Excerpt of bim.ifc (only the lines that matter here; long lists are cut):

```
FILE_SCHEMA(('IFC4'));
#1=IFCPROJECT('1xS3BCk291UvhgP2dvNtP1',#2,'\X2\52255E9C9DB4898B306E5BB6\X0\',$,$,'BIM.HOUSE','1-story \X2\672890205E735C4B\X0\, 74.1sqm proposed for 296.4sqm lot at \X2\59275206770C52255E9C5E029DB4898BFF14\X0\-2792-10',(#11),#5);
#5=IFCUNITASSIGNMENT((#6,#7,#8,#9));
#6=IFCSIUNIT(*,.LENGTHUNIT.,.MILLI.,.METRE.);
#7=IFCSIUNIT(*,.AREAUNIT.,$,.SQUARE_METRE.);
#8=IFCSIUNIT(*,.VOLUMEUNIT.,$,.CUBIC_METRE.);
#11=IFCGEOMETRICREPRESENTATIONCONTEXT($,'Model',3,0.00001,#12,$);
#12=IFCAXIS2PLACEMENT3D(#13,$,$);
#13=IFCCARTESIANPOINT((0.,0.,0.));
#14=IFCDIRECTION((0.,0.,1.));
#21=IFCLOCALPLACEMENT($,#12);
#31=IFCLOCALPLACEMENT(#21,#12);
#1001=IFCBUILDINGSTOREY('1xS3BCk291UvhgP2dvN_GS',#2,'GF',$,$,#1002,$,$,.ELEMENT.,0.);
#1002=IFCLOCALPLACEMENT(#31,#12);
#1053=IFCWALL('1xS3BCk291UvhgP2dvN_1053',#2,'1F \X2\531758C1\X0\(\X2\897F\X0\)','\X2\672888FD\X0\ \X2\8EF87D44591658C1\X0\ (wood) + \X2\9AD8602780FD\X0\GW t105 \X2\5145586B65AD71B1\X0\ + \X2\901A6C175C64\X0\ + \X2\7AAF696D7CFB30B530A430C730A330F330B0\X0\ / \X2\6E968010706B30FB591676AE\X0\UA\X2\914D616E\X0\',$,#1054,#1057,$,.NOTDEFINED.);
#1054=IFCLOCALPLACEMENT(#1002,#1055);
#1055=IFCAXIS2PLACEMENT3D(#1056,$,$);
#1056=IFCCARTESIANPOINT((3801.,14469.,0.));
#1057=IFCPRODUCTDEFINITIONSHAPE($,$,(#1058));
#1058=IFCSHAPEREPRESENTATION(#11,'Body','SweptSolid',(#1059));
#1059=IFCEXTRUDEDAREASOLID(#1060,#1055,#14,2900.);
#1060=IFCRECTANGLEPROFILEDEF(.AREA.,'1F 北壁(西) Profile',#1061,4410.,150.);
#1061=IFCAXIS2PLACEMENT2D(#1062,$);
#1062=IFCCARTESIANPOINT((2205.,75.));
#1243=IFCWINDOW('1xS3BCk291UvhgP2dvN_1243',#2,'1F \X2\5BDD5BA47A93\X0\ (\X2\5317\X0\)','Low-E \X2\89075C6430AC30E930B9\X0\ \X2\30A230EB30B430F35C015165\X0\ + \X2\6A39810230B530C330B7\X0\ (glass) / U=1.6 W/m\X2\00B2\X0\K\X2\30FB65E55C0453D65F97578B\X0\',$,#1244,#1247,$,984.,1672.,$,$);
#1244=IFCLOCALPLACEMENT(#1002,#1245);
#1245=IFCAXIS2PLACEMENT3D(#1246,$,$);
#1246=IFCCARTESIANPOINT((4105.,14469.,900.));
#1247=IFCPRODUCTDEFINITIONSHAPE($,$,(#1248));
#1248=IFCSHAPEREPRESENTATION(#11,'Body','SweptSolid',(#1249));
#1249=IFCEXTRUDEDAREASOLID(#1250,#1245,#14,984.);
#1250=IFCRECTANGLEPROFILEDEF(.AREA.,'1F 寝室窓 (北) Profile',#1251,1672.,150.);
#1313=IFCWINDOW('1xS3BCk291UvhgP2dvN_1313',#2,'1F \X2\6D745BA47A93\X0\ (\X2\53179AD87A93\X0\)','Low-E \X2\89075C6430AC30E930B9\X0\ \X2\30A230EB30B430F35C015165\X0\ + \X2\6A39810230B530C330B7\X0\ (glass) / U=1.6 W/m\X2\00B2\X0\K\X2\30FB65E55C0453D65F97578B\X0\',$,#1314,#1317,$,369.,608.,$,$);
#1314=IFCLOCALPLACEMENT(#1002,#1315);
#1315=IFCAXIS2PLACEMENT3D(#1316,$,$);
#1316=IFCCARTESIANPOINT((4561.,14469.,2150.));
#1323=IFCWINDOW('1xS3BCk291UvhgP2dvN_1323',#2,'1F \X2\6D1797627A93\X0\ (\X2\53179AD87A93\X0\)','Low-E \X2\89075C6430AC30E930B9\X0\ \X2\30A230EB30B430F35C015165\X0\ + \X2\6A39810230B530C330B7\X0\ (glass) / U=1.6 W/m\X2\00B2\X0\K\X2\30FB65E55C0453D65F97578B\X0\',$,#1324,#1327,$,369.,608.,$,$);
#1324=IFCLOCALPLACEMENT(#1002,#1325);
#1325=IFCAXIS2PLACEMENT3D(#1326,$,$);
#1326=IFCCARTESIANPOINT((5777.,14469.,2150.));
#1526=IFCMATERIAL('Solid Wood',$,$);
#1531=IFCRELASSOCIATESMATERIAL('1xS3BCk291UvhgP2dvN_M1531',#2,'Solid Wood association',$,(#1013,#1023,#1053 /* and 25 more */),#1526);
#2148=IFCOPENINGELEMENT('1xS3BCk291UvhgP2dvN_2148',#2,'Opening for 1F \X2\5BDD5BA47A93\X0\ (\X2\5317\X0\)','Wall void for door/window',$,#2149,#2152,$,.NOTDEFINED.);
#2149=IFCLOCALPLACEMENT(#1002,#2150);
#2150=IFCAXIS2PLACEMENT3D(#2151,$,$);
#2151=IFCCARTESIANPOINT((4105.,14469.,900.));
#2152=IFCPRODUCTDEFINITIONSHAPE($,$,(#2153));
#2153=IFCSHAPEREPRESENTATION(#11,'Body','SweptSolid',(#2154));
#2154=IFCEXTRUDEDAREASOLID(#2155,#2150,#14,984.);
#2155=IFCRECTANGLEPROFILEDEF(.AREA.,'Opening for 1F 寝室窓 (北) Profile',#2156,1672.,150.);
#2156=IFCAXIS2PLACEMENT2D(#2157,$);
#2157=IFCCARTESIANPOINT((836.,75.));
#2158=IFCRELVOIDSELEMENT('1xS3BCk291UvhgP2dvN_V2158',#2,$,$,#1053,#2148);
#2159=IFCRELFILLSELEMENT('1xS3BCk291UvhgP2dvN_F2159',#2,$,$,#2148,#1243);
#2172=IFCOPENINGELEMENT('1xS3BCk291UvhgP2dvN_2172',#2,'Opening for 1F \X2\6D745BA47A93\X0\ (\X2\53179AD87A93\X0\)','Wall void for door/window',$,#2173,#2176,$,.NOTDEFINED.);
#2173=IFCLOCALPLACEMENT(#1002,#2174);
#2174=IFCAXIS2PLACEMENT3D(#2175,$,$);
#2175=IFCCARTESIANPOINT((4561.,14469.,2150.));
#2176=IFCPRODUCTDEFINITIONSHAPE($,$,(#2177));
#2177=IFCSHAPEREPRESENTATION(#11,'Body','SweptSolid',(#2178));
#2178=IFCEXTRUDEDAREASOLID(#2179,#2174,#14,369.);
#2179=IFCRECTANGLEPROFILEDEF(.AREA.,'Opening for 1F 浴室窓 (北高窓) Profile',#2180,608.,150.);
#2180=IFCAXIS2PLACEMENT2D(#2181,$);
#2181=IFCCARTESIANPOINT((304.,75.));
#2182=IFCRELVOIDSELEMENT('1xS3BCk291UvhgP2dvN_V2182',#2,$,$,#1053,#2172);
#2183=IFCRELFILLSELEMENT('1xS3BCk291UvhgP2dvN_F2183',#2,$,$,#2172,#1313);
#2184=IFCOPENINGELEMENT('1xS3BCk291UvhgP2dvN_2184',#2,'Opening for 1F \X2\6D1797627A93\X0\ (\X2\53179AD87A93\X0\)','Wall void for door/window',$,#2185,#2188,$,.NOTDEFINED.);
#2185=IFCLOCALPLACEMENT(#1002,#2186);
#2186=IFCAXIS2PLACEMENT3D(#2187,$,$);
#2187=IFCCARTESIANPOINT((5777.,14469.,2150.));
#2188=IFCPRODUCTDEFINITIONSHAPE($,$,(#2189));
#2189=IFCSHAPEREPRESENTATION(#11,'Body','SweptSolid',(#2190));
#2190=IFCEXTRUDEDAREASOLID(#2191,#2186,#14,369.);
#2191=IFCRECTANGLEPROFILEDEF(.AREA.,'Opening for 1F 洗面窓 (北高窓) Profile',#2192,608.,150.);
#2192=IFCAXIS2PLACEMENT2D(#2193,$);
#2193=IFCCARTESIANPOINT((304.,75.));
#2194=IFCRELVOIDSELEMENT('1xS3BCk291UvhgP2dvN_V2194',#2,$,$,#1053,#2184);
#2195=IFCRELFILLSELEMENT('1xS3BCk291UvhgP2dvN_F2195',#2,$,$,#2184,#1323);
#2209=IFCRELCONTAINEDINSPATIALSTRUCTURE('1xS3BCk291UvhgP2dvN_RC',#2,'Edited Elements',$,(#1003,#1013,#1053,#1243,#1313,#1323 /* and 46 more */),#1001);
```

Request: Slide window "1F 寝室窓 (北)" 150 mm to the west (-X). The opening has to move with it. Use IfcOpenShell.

```python
import ifcopenshell
import ifcopenshell.api.geometry
import ifcopenshell.util.placement

model = ifcopenshell.open("bim.ifc")

window = model.by_guid("1xS3BCk291UvhgP2dvN_1243")
opening = window.FillsVoids[0].RelatingOpeningElement
wall = opening.VoidsElements[0].RelatingBuildingElement

wall_matrix = ifcopenshell.util.placement.get_local_placement(wall.ObjectPlacement)
shift = wall_matrix[:3, 0] * -150.0
before = ifcopenshell.util.placement.get_local_placement(window.ObjectPlacement)[:3, 3].copy()

# The window is not placed relative to its opening, so move both.
for product in (opening, window):
    matrix = ifcopenshell.util.placement.get_local_placement(product.ObjectPlacement)
    matrix[:3, 3] += shift
    ifcopenshell.api.geometry.edit_object_placement(model, product=product, matrix=matrix, is_si=False)

after = ifcopenshell.util.placement.get_local_placement(window.ObjectPlacement)[:3, 3]
print("window moved by", (after - before).round(3) + 0.0)

model.write("bim_edited.ifc")
```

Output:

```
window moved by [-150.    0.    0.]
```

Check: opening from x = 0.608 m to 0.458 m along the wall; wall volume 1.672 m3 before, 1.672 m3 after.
